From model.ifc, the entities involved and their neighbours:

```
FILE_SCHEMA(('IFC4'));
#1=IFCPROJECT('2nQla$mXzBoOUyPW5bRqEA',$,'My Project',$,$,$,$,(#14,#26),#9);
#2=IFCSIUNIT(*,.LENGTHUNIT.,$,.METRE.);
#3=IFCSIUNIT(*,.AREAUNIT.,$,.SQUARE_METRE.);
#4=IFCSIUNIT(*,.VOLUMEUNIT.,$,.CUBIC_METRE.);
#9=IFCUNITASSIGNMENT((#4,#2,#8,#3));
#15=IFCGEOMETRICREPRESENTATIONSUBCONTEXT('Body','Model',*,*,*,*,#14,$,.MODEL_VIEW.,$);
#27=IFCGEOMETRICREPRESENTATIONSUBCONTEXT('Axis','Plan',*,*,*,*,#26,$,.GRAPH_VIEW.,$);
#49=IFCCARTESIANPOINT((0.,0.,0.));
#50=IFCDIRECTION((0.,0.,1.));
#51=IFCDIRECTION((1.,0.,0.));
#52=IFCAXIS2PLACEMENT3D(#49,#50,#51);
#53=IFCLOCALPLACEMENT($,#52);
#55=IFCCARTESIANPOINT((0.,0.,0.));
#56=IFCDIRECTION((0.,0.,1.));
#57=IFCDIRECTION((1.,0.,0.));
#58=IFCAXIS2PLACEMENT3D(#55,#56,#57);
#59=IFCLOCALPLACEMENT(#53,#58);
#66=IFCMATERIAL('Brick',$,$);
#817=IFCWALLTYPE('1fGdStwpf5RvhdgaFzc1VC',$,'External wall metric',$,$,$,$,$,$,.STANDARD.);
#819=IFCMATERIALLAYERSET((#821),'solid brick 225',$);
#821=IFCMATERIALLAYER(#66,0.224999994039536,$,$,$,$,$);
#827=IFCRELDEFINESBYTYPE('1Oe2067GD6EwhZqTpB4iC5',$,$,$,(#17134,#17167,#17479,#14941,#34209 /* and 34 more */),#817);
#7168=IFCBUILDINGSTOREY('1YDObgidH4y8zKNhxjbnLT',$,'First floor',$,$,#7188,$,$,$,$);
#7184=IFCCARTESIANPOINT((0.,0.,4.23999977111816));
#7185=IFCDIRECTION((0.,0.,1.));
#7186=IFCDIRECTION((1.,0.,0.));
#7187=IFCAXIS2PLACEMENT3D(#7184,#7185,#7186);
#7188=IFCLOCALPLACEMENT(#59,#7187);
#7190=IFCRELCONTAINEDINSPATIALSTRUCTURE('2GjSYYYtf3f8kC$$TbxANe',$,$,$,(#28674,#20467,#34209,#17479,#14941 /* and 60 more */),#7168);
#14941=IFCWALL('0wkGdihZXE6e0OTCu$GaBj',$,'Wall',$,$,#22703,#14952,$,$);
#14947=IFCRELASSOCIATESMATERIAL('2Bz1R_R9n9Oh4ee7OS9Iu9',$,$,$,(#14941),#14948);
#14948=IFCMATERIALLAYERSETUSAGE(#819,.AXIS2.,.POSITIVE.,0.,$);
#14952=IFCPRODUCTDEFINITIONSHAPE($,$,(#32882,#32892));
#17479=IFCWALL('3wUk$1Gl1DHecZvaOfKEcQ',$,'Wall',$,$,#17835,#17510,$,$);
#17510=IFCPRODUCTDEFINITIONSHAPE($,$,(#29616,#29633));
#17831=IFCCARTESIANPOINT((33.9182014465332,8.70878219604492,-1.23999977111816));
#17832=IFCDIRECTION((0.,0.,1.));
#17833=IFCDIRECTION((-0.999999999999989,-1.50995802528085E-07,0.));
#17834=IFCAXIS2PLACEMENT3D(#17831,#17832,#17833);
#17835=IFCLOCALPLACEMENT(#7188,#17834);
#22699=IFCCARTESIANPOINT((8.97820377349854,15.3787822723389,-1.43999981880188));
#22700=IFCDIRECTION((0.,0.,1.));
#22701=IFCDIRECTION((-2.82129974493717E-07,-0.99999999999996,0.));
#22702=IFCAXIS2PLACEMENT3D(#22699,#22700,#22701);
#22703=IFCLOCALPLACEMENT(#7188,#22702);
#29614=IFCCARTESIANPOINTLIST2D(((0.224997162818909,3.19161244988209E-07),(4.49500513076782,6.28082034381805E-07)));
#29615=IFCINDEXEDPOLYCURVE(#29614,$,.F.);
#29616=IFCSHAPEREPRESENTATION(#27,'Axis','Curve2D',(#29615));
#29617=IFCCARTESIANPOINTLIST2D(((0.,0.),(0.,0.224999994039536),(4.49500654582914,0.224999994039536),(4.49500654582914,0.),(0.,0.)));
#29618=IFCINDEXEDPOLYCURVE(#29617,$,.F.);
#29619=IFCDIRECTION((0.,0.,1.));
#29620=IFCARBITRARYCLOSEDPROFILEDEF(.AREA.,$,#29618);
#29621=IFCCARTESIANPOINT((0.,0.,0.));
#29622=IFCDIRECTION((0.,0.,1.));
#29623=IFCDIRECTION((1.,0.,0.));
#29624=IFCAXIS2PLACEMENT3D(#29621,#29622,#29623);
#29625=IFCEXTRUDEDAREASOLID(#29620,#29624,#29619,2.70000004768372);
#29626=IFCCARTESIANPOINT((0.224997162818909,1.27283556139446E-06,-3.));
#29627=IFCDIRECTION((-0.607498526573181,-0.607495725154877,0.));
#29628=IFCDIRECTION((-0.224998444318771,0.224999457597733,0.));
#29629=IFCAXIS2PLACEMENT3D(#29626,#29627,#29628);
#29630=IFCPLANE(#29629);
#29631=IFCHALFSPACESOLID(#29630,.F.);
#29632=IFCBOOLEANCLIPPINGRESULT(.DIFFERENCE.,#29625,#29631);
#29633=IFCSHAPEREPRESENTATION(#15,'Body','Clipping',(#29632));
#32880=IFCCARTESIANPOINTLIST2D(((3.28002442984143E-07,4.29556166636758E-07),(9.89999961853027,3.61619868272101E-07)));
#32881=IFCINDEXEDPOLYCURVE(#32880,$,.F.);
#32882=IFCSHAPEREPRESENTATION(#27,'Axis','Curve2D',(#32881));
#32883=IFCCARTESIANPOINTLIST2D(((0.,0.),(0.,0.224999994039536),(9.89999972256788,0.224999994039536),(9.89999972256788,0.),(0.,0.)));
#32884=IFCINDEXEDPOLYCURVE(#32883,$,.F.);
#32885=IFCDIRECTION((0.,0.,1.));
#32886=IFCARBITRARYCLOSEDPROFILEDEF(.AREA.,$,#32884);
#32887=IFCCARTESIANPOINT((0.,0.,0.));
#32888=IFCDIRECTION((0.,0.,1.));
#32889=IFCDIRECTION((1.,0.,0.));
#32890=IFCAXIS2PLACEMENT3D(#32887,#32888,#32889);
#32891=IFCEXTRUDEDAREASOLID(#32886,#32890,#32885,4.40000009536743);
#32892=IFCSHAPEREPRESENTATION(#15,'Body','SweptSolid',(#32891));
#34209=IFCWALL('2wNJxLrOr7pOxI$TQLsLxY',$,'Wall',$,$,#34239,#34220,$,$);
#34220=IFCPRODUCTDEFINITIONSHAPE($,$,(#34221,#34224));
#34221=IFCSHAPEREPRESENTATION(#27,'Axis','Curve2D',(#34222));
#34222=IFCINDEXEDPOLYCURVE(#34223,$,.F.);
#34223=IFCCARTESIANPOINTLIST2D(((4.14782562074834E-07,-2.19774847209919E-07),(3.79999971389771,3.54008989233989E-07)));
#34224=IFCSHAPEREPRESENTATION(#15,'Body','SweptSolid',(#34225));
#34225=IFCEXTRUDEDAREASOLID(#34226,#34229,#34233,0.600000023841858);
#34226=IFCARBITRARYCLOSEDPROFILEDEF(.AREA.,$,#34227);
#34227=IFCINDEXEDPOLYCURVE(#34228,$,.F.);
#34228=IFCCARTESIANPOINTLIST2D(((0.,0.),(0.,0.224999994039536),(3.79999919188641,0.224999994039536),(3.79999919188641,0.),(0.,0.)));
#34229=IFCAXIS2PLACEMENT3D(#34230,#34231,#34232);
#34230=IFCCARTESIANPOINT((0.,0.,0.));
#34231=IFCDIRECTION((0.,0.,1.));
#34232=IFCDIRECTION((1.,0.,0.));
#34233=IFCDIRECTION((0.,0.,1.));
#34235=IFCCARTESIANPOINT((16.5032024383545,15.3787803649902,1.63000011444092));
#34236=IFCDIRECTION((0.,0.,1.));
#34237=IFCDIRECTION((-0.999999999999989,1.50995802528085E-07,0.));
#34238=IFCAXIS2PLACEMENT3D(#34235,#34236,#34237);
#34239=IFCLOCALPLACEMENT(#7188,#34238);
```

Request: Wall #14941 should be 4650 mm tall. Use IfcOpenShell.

```python
import ifcopenshell
import ifcopenshell.geom
import ifcopenshell.util.representation
import ifcopenshell.util.shape
import ifcopenshell.util.unit

model = ifcopenshell.open("model.ifc")
unit_scale = ifcopenshell.util.unit.calculate_unit_scale(model)
settings = ifcopenshell.geom.settings()


def volume(element):
    """Net volume in cubic metres, openings subtracted."""
    shape = ifcopenshell.geom.create_shape(settings, element)
    return ifcopenshell.util.shape.get_volume(shape.geometry)


wall = model.by_guid("0wkGdihZXE6e0OTCu$GaBj")
before = volume(wall)

body = ifcopenshell.util.representation.get_representation(wall, "Model", "Body")
solid = body.Items[0]
old_height = solid.Depth
solid.Depth = 4.65 / unit_scale
after = volume(wall)

print(f"height {old_height:g} -> {solid.Depth:g}, volume {before:.3f} -> {after:.3f} m3")

model.write("model-out.ifc")
```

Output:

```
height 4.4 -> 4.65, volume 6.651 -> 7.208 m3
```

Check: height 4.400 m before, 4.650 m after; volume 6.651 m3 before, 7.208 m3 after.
